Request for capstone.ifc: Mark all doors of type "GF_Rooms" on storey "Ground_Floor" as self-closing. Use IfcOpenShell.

First a look at what the model holds.

```python
import ifcopenshell
import ifcopenshell.util.element

model = ifcopenshell.open("capstone.ifc")
print(model.schema)
storey = next(s for s in model.by_type("IfcBuildingStorey") if s.Name == "Ground_Floor")
doors = [e for e in ifcopenshell.util.element.get_decomposition(storey) if e.is_a("IfcDoor")]
seen = {}
for e in doors:
    element_type = ifcopenshell.util.element.get_type(e)
    key = (element_type.Name if element_type != e and element_type else None, ifcopenshell.util.element.get_pset(e, "Pset_DoorCommon", "SelfClosing"))
    seen[key] = seen.get(key, 0) + 1
for (name, value), count in sorted(seen.items(), key=str):
    print(count, "x", name, "|", value)
```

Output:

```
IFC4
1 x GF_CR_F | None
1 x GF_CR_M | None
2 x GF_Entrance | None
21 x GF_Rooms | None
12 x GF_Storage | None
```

```python
import ifcopenshell
import ifcopenshell.api.pset
import ifcopenshell.util.element

model = ifcopenshell.open("capstone.ifc")

storey = next(s for s in model.by_type("IfcBuildingStorey") if s.Name == "Ground_Floor")
doors = [e for e in ifcopenshell.util.element.get_decomposition(storey) if e.is_a("IfcDoor")]

count = 0
for e in doors:
    element_type = ifcopenshell.util.element.get_type(e)
    if element_type in (None, e) or element_type.Name != "GF_Rooms":
        continue
    # add_pset returns the element's existing set when there is one.
    pset = ifcopenshell.api.pset.add_pset(model, product=e, name="Pset_DoorCommon")
    ifcopenshell.api.pset.edit_pset(model, pset=pset, properties={"SelfClosing": True})
    count += 1

print(count, "doors updated")

model.write("capstone_updated.ifc")
```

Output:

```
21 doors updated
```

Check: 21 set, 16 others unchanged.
